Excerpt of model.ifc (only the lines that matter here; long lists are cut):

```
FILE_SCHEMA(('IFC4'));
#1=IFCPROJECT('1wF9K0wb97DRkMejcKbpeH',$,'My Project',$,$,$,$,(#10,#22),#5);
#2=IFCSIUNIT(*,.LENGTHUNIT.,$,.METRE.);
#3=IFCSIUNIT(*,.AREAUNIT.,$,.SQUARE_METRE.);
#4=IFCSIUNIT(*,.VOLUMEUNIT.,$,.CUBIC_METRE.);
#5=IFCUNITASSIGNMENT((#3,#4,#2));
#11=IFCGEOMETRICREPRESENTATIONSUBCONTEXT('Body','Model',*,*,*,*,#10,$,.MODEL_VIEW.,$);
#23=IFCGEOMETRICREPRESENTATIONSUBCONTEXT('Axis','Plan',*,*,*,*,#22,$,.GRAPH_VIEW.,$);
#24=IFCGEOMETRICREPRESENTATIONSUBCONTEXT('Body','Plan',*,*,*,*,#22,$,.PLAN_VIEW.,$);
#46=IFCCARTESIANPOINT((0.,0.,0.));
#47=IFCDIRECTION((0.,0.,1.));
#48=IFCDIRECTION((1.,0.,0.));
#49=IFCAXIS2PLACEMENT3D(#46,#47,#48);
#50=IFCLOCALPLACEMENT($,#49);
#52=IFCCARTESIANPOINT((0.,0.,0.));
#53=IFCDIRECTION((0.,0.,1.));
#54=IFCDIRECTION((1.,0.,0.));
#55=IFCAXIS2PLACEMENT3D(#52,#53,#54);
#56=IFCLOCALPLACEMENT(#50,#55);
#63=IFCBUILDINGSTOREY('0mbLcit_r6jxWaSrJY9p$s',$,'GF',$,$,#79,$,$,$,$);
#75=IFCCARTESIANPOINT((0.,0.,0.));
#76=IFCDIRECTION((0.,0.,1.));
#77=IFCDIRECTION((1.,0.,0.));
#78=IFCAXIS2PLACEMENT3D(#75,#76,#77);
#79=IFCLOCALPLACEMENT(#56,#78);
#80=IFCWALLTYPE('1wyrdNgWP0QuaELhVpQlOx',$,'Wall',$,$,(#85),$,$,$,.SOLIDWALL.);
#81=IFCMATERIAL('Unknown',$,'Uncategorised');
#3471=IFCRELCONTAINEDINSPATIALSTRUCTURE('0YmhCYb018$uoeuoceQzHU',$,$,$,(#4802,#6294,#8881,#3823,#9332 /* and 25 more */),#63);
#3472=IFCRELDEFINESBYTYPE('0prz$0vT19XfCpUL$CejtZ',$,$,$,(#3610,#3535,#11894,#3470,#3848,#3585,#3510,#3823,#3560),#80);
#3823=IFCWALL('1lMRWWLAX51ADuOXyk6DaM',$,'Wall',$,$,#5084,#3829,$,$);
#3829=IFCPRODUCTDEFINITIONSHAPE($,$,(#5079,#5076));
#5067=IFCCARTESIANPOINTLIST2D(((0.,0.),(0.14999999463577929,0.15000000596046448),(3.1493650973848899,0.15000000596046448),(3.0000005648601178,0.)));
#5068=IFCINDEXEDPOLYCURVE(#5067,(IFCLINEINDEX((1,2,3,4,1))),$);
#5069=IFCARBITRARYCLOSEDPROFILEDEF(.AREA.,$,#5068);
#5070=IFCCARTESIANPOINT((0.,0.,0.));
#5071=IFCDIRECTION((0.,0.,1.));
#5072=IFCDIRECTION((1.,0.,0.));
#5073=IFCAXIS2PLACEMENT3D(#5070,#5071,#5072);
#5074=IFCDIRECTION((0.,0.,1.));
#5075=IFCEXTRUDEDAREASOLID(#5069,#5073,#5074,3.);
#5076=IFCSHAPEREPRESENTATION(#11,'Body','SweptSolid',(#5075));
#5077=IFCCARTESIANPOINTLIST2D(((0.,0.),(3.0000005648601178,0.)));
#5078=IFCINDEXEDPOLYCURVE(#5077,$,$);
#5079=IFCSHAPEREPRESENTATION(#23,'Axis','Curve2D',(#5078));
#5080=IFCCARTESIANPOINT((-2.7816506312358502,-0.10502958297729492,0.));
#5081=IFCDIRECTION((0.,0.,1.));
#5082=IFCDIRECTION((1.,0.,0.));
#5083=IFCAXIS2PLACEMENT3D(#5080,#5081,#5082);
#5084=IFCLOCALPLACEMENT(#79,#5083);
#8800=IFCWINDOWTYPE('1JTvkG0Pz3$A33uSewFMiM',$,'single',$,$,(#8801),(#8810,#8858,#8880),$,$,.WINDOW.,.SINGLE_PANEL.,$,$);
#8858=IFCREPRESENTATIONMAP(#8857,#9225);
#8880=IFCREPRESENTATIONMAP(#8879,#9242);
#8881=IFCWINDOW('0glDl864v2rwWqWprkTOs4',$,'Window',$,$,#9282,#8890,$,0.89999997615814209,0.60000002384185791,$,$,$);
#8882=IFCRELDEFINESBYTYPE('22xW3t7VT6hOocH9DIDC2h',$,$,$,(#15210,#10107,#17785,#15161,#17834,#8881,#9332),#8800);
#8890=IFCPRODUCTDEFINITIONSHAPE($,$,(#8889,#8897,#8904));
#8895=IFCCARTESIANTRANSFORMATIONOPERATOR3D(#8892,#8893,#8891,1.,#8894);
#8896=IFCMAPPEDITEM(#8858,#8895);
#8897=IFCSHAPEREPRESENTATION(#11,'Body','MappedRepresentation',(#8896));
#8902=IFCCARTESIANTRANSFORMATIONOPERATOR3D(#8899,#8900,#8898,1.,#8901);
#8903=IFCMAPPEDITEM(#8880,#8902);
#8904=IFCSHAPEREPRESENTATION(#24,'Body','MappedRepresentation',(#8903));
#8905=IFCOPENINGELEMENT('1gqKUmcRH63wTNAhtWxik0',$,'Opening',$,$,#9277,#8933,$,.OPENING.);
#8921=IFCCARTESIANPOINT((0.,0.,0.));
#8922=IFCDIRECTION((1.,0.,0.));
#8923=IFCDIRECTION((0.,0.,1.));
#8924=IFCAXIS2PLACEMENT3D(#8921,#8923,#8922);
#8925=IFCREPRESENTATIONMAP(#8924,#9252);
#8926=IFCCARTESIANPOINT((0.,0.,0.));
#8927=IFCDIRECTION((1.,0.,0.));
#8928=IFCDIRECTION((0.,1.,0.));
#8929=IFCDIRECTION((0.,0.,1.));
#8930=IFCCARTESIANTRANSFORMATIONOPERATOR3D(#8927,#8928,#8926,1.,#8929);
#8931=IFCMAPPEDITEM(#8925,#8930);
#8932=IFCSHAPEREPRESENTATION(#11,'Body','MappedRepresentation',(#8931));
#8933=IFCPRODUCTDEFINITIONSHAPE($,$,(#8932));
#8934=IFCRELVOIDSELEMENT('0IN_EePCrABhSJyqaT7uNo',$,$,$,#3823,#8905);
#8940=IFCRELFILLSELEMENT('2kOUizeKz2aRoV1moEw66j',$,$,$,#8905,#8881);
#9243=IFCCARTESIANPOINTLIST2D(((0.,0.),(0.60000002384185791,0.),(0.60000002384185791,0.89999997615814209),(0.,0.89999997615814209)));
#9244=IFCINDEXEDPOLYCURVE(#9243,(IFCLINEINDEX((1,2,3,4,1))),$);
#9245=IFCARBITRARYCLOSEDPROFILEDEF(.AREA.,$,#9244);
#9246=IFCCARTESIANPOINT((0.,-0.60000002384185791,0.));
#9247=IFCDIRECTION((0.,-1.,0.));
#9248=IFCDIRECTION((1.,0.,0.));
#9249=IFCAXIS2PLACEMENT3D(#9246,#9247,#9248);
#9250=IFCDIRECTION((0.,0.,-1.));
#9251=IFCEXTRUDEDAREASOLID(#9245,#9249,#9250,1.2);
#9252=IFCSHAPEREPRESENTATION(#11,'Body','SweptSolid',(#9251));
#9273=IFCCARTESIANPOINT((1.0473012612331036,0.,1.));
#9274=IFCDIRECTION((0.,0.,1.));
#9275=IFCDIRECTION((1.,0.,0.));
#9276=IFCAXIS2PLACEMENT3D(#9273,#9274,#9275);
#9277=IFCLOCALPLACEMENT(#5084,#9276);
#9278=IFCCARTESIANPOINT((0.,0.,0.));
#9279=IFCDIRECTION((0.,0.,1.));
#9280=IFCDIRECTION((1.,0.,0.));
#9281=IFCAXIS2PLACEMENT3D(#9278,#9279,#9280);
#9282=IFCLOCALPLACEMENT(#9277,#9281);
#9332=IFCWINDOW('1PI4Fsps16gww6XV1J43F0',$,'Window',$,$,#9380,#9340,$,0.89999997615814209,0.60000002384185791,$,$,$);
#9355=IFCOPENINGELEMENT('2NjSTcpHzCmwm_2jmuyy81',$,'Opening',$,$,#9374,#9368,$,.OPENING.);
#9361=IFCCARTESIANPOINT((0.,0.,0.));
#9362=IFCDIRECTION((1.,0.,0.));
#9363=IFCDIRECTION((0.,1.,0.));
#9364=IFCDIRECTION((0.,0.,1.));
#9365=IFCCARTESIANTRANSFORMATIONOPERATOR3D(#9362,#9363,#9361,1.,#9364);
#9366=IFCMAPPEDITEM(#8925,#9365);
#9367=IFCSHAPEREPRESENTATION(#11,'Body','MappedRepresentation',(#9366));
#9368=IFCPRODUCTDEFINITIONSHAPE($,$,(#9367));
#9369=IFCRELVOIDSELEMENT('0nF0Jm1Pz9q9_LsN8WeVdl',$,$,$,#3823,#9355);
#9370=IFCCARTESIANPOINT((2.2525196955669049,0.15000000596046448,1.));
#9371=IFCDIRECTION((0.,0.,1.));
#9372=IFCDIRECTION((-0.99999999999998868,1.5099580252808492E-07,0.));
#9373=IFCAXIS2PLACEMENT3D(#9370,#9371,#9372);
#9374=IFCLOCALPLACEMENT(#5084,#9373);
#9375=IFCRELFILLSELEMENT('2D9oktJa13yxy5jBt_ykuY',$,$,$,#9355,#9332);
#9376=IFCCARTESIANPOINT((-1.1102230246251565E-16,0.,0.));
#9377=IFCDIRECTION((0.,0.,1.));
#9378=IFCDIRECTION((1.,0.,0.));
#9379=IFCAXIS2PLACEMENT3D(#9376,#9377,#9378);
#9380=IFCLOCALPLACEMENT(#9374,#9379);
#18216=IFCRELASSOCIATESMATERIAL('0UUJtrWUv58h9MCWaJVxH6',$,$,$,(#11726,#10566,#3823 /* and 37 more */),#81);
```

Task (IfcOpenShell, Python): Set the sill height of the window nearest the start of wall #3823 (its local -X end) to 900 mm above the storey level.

```python
import numpy as np
import ifcopenshell
import ifcopenshell.api.geometry
import ifcopenshell.geom
import ifcopenshell.util.element
import ifcopenshell.util.placement
import ifcopenshell.util.shape
import ifcopenshell.util.unit

model = ifcopenshell.open("model.ifc")
unit_scale = ifcopenshell.util.unit.calculate_unit_scale(model)

window = model.by_id(8881)
opening = window.FillsVoids[0].RelatingOpeningElement
storey = ifcopenshell.util.element.get_container(window, ifc_class="IfcBuildingStorey")
level = ifcopenshell.util.placement.get_local_placement(storey.ObjectPlacement)[2, 3]

# The opening's origin need not be at the sill, so measure its lowest point.
shape = ifcopenshell.geom.create_shape(ifcopenshell.geom.settings(), opening)
bottom = ifcopenshell.util.shape.get_shape_bottom_elevation(shape, shape.geometry) / unit_scale
dz = level + 0.9 / unit_scale - bottom

shift = np.array([0.0, 0.0, dz])
# The window is placed relative to its opening, so it follows when the opening moves.
matrix = ifcopenshell.util.placement.get_local_placement(opening.ObjectPlacement)
matrix[:3, 3] += shift
ifcopenshell.api.geometry.edit_object_placement(
    model, product=opening, matrix=matrix, is_si=False, should_transform_children=True
)

print(f"moved by {dz * unit_scale:+.3f} m")

model.write("model-out.ifc")
```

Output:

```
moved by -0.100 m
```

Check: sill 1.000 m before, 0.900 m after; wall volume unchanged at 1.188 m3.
